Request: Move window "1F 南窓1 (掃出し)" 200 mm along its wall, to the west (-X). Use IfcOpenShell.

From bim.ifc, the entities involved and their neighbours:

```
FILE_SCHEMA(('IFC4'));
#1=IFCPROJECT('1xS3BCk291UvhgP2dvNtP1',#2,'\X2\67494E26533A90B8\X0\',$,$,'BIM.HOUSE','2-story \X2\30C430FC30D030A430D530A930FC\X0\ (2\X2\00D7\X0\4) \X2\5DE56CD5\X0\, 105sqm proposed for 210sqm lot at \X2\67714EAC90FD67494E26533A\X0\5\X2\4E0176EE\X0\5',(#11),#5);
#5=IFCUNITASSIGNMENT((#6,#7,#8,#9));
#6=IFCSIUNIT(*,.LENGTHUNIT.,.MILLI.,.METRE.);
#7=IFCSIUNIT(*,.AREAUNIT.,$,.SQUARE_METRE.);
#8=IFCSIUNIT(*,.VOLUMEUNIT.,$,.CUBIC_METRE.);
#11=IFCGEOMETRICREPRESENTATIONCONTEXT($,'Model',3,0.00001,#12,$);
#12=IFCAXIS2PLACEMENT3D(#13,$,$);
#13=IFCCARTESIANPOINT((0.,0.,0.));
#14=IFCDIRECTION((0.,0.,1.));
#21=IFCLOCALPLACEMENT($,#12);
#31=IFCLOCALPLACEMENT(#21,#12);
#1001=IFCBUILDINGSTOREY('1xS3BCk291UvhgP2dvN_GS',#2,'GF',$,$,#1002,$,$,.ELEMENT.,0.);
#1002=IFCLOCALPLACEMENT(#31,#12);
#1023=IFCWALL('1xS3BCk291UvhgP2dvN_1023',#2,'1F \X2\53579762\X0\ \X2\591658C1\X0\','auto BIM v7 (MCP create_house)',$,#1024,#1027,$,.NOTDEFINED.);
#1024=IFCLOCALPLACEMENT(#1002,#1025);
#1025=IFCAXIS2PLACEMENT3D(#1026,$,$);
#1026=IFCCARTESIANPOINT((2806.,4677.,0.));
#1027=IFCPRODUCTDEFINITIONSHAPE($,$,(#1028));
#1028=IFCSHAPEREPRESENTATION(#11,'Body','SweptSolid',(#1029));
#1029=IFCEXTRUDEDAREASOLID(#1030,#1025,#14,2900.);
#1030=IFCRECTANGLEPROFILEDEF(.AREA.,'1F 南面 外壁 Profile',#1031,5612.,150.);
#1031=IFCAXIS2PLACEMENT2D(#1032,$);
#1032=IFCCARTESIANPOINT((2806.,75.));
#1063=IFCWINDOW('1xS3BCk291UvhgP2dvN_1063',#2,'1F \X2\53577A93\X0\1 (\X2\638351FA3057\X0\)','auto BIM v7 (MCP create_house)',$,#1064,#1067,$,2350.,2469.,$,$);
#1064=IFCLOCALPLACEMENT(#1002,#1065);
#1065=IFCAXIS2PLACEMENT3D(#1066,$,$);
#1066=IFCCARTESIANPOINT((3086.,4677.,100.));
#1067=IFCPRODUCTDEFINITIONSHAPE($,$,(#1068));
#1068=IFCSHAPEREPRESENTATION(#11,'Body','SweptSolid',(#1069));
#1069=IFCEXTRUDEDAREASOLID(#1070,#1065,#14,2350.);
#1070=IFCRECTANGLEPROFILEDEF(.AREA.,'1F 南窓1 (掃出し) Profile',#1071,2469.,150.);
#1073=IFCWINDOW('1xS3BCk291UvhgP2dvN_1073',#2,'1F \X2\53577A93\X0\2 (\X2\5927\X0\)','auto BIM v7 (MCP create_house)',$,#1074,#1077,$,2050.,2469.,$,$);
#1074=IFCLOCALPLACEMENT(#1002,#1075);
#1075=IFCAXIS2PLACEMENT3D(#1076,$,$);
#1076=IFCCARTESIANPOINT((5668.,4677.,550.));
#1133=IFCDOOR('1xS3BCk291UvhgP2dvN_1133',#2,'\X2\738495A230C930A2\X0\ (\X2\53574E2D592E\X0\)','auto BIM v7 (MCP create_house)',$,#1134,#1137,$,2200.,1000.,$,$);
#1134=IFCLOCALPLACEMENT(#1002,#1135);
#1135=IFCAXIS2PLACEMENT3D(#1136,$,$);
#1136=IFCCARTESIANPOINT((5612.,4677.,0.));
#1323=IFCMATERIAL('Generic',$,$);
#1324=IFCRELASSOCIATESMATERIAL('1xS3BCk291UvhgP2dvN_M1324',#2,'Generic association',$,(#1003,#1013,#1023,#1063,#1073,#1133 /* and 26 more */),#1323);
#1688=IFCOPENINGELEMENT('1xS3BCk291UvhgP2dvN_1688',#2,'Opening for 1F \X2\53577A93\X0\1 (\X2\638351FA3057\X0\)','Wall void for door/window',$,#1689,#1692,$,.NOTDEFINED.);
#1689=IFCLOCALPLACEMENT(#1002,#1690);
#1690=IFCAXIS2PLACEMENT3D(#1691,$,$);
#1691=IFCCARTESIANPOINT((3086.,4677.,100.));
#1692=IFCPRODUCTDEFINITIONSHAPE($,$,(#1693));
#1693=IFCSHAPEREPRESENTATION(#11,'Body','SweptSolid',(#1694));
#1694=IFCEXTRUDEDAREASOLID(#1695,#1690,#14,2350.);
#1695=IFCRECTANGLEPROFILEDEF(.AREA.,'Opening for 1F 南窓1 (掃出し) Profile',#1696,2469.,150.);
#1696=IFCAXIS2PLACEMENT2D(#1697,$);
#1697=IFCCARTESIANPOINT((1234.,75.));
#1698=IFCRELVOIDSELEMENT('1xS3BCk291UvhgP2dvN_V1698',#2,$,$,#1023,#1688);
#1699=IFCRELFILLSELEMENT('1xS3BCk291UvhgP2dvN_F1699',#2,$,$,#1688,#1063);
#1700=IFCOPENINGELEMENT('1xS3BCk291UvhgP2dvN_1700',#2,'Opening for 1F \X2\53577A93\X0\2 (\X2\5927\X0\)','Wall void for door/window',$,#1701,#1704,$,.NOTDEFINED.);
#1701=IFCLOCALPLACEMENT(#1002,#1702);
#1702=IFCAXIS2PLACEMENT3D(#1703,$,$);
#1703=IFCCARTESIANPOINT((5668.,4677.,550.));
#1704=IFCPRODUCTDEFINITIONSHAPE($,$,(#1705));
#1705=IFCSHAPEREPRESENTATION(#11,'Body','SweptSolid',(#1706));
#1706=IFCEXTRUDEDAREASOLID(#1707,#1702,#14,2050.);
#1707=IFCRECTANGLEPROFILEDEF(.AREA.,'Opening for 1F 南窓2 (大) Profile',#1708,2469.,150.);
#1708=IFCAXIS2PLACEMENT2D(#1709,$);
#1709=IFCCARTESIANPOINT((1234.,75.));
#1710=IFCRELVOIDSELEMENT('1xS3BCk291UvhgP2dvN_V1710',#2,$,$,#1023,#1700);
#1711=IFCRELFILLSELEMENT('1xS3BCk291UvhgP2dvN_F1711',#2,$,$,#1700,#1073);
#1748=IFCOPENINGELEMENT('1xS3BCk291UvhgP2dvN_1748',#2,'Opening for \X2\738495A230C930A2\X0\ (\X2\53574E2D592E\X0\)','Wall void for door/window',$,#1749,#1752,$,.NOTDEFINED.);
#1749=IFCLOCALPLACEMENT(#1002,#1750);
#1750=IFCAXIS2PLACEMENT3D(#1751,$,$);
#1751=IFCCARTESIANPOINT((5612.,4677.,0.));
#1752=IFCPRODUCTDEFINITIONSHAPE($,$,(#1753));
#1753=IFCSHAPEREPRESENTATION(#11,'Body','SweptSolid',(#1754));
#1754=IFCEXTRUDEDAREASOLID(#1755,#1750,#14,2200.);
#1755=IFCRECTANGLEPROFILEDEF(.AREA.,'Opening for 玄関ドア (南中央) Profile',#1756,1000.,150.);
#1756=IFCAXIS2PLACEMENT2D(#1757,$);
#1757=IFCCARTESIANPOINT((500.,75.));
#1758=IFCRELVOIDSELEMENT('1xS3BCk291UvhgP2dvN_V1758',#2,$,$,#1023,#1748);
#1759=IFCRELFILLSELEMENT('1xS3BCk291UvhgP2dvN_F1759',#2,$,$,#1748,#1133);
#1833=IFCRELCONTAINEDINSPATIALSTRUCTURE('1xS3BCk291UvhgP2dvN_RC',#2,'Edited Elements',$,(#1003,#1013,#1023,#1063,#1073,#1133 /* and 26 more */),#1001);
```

```python
import ifcopenshell
import ifcopenshell.api.geometry
import ifcopenshell.util.placement
import ifcopenshell.util.unit

model = ifcopenshell.open("bim.ifc")
unit_scale = ifcopenshell.util.unit.calculate_unit_scale(model)

window = model.by_guid("1xS3BCk291UvhgP2dvN_1063")
opening = window.FillsVoids[0].RelatingOpeningElement
wall = opening.VoidsElements[0].RelatingBuildingElement

wall_matrix = ifcopenshell.util.placement.get_local_placement(wall.ObjectPlacement)
shift = wall_matrix[:3, 0] * -0.2 / unit_scale
before = ifcopenshell.util.placement.get_local_placement(window.ObjectPlacement)[:3, 3].copy()

# The window is not placed relative to its opening, so move both.
for product in (opening, window):
    matrix = ifcopenshell.util.placement.get_local_placement(product.ObjectPlacement)
    matrix[:3, 3] += shift
    ifcopenshell.api.geometry.edit_object_placement(model, product=product, matrix=matrix, is_si=False)

after = ifcopenshell.util.placement.get_local_placement(window.ObjectPlacement)[:3, 3]
print("window moved by", (after - before).round(3) + 0.0)

model.write("bim_updated.ifc")
```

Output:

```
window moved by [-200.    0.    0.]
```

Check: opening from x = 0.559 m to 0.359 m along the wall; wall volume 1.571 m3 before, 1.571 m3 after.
